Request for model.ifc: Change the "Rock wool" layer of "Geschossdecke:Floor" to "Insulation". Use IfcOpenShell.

First a look at what the model holds.

```python
import ifcopenshell
import ifcopenshell.util.element

model = ifcopenshell.open("model.ifc")
print(model.schema)
for layer_set in model.by_type("IfcMaterialLayerSet"):
    if layer_set.LayerSetName == "Geschossdecke:Floor":
        for layer in layer_set.MaterialLayers:
            print(layer.id(), layer.Material and layer.Material.Name, layer.LayerThickness, sep=" | ")
        print(len(ifcopenshell.util.element.get_elements_by_material(model, layer_set)), "elements and types use it")
print(sorted(m.Name for m in model.by_type("IfcMaterial") if m.Name)[:60])
```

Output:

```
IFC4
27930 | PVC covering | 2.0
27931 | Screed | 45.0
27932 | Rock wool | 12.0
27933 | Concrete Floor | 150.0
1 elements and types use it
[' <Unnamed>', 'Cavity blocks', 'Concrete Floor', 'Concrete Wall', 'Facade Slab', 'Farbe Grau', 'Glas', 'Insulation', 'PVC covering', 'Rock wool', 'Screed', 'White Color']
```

```python
import ifcopenshell
import ifcopenshell.api.material

model = ifcopenshell.open("model.ifc")

layer_set = next(s for s in model.by_type("IfcMaterialLayerSet") if s.LayerSetName == "Geschossdecke:Floor")
layer = next(l for l in layer_set.MaterialLayers if l.Material and l.Material.Name == "Rock wool")
material = next(m for m in model.by_type("IfcMaterial") if m.Name == "Insulation")

# Point this one layer at the other material; renaming the old one would change it everywhere.
ifcopenshell.api.material.edit_layer(model, layer=layer, attributes={}, material=material)

print([l.Material.Name if l.Material else None for l in layer_set.MaterialLayers])

model.write("model_updated.ifc")
```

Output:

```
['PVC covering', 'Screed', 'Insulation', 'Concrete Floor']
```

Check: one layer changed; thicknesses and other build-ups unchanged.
